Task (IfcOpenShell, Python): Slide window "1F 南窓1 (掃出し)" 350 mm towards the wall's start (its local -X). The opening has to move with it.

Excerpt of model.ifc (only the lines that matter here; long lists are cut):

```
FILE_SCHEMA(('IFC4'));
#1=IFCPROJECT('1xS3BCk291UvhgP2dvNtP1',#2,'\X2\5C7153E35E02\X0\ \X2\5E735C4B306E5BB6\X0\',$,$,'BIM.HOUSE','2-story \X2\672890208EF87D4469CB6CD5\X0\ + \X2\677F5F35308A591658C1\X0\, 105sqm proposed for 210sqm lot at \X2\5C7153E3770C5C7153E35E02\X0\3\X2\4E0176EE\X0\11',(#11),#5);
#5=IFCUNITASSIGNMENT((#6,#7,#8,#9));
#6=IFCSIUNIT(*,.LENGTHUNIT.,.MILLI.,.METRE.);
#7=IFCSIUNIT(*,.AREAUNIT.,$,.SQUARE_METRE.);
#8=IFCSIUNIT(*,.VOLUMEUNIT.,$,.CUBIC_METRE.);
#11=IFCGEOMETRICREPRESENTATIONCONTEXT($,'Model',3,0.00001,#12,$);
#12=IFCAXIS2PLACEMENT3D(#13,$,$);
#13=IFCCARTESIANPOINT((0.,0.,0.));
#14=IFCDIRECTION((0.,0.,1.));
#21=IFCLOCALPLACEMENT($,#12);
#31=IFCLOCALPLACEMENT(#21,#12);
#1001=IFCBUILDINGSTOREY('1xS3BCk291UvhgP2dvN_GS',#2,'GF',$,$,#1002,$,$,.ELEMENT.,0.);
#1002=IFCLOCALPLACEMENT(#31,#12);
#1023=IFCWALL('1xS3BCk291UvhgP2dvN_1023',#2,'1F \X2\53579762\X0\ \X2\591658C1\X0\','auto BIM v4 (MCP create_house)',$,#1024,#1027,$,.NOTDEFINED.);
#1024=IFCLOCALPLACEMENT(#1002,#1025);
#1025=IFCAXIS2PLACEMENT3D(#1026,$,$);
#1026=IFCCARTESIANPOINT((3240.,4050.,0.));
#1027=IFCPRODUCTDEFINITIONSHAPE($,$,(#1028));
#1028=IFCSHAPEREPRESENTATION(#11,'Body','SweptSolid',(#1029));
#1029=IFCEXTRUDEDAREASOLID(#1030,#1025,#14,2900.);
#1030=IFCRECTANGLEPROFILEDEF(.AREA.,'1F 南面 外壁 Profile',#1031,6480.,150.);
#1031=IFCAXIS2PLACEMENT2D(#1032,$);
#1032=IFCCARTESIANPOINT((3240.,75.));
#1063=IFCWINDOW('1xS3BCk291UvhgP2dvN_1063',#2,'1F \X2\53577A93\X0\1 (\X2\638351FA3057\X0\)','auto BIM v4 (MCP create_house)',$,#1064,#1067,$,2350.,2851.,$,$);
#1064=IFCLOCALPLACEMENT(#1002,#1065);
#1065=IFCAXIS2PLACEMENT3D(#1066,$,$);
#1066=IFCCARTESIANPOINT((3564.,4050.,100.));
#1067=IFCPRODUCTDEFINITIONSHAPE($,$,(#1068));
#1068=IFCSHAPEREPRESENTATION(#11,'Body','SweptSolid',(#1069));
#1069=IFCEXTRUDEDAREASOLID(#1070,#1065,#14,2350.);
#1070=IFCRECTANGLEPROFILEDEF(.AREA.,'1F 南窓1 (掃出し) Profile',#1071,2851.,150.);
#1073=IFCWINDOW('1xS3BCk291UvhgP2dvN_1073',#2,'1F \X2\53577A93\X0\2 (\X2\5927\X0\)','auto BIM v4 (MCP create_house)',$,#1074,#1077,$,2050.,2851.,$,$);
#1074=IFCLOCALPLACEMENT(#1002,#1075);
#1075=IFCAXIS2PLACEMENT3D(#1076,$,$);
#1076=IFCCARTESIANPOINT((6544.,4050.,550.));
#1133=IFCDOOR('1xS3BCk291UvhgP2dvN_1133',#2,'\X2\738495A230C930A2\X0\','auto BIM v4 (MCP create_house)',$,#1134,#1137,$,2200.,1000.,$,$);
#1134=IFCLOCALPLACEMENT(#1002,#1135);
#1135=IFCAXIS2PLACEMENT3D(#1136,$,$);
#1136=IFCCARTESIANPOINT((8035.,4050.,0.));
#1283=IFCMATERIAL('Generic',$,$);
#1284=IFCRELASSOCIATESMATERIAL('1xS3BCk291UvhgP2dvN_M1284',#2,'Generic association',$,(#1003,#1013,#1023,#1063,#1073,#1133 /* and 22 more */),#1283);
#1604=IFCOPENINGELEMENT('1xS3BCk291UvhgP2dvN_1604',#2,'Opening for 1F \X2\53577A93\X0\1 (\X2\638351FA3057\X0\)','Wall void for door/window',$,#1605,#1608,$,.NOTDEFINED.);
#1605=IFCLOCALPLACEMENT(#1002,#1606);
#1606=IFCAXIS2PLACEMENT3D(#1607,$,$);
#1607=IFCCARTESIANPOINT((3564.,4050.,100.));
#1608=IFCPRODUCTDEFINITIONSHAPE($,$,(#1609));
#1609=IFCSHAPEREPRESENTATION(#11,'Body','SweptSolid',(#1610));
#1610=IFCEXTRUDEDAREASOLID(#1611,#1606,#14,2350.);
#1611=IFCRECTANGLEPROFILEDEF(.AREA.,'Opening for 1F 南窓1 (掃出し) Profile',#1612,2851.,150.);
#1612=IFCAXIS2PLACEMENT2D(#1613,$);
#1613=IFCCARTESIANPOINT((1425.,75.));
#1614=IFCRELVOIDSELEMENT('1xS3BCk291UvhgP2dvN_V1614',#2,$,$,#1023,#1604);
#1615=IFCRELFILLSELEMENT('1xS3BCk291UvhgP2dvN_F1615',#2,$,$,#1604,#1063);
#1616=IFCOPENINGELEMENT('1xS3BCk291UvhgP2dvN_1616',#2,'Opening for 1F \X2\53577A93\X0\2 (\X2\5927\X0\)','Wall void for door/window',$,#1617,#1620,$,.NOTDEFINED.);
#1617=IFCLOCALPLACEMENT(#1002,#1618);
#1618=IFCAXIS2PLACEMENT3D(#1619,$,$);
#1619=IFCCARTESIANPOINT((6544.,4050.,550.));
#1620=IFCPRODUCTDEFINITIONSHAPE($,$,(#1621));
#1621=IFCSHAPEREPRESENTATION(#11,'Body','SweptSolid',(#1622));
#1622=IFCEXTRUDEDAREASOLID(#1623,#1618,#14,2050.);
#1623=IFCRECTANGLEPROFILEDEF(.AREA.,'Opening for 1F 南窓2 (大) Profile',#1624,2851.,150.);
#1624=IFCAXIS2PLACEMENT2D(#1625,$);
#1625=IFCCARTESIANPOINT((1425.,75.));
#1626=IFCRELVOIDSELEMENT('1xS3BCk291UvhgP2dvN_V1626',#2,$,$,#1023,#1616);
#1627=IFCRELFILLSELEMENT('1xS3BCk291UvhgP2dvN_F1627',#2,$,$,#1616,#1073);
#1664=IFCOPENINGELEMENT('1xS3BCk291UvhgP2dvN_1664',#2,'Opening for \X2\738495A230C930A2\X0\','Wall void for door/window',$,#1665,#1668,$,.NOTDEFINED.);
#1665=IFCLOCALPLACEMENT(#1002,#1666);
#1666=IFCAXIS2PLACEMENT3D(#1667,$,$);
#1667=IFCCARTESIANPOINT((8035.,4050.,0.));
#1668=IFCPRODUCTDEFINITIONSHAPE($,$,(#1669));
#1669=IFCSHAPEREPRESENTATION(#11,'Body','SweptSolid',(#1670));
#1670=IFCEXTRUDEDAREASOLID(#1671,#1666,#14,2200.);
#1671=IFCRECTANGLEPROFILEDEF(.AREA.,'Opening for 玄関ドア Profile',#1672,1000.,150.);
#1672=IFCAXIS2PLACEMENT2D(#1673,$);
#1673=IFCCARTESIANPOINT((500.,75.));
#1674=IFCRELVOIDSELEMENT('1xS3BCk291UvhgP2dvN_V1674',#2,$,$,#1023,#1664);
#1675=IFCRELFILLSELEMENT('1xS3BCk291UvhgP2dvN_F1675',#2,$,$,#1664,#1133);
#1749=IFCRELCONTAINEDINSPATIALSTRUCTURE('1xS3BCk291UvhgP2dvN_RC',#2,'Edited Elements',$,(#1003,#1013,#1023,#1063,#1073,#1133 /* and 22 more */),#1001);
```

```python
import ifcopenshell
import ifcopenshell.api.geometry
import ifcopenshell.util.placement

model = ifcopenshell.open("model.ifc")

window = model.by_guid("1xS3BCk291UvhgP2dvN_1063")
opening = window.FillsVoids[0].RelatingOpeningElement
wall = opening.VoidsElements[0].RelatingBuildingElement

wall_matrix = ifcopenshell.util.placement.get_local_placement(wall.ObjectPlacement)
shift = wall_matrix[:3, 0] * -350.0
before = ifcopenshell.util.placement.get_local_placement(window.ObjectPlacement)[:3, 3].copy()

# The window is not placed relative to its opening, so move both.
for product in (opening, window):
    matrix = ifcopenshell.util.placement.get_local_placement(product.ObjectPlacement)
    matrix[:3, 3] += shift
    ifcopenshell.api.geometry.edit_object_placement(model, product=product, matrix=matrix, is_si=False)

after = ifcopenshell.util.placement.get_local_placement(window.ObjectPlacement)[:3, 3]
print("window moved by", (after - before).round(3) + 0.0)

model.write("model_edited.ifc")
```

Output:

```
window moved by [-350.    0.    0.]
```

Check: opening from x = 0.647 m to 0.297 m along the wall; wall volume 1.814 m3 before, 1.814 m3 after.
